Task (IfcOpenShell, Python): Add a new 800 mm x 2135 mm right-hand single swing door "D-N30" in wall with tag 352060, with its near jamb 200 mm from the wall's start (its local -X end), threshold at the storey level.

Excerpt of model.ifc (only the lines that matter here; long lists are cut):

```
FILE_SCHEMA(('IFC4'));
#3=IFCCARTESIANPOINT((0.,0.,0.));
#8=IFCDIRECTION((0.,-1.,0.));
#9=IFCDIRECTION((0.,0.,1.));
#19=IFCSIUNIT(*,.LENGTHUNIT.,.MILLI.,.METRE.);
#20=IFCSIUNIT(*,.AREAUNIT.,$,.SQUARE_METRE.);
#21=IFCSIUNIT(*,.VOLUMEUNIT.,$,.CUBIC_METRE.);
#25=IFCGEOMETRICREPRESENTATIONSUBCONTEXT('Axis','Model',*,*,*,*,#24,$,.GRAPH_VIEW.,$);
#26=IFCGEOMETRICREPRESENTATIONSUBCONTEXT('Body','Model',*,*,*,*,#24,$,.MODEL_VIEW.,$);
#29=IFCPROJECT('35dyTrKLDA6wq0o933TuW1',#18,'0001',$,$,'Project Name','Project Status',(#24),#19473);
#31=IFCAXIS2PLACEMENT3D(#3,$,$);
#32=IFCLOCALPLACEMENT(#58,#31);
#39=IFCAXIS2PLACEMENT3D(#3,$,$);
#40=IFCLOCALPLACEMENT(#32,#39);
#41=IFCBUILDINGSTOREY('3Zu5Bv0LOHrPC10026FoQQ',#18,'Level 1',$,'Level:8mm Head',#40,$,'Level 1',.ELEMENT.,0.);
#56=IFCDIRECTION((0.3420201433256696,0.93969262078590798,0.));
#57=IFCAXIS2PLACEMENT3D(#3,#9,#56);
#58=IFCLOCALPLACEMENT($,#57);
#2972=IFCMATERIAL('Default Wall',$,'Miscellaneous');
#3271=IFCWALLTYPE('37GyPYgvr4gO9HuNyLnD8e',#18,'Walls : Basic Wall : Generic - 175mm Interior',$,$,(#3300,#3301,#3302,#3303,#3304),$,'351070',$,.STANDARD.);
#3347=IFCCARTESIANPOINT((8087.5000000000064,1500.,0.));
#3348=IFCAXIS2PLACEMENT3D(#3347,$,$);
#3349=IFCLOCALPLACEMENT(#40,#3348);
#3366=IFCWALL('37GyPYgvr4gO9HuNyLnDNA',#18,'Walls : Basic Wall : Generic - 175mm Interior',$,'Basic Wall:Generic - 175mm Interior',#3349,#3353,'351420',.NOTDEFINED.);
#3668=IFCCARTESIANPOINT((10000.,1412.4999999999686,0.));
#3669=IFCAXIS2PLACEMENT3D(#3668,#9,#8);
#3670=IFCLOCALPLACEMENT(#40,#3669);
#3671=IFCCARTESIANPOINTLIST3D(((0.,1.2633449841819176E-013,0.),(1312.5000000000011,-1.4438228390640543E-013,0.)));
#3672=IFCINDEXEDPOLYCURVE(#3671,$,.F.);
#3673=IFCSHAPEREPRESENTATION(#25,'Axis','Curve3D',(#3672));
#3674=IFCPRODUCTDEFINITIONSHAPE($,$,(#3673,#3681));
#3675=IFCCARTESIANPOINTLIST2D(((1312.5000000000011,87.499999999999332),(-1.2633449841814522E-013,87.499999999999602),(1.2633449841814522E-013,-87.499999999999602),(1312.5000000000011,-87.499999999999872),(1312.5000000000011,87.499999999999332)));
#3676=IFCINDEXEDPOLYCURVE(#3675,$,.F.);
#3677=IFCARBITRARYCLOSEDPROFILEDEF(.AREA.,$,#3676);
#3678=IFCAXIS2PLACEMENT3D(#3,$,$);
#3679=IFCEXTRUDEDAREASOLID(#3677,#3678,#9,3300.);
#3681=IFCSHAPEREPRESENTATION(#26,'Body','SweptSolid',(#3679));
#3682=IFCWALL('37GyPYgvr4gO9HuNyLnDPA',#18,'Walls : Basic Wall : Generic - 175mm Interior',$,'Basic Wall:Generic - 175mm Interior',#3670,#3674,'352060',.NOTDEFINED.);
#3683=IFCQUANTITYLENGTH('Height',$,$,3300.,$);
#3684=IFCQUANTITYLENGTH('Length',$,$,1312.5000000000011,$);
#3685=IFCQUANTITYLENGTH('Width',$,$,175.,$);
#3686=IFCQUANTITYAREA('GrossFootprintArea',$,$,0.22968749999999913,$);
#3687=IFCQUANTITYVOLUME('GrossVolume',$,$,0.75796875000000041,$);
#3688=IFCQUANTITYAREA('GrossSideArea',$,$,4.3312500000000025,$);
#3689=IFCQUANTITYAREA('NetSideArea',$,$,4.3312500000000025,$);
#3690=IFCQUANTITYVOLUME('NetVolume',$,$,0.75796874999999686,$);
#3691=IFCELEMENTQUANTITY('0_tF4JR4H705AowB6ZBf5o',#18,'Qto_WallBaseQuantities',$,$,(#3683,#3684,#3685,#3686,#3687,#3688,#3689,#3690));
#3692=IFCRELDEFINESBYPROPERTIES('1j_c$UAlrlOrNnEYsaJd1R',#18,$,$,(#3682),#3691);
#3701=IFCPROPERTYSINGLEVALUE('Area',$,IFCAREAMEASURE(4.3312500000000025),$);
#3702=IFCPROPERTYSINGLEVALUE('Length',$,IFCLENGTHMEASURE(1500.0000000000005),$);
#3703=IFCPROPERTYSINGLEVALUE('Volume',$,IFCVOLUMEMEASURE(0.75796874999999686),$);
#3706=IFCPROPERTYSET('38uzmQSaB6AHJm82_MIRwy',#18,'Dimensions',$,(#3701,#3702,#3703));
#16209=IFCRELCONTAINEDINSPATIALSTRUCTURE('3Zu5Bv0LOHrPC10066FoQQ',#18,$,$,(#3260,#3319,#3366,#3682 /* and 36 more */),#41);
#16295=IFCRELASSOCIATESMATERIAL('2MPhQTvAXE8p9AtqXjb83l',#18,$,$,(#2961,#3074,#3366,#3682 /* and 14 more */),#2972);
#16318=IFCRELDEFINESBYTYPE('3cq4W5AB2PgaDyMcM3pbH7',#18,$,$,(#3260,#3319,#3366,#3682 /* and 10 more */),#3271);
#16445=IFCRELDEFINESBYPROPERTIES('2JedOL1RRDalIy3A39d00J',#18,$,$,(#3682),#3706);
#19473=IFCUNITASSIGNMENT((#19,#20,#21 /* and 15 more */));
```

```python
import numpy as np
import ifcopenshell
import ifcopenshell.api.feature
import ifcopenshell.api.geometry
import ifcopenshell.api.pset
import ifcopenshell.api.root
import ifcopenshell.api.spatial
import ifcopenshell.geom
import ifcopenshell.util.element
import ifcopenshell.util.placement
import ifcopenshell.util.representation
import ifcopenshell.util.shape
import ifcopenshell.util.unit

model = ifcopenshell.open("model.ifc")
unit_scale = ifcopenshell.util.unit.calculate_unit_scale(model)
area_scale = ifcopenshell.util.unit.calculate_unit_scale(model, "AREAUNIT")
volume_scale = ifcopenshell.util.unit.calculate_unit_scale(model, "VOLUMEUNIT")
settings = ifcopenshell.geom.settings()


def volume(element):
    """Net volume in cubic metres, openings subtracted."""
    shape = ifcopenshell.geom.create_shape(settings, element)
    return ifcopenshell.util.shape.get_volume(shape.geometry)


wall = model.by_guid("37GyPYgvr4gO9HuNyLnDPA")
storey = ifcopenshell.util.element.get_container(wall, ifc_class="IfcBuildingStorey")
context = ifcopenshell.util.representation.get_context(model, "Model", "Body", "MODEL_VIEW")
before = volume(wall)

width, height, from_end, sill = 0.8, 2.135, 0.2, 0.0  # metres

# The wall runs along its own X axis, and the end named is its -X end.
wall_shape = ifcopenshell.geom.create_shape(settings, wall)
x, y, z = ifcopenshell.util.shape.get_vertices(wall_shape.geometry).T
start = x.min() + from_end
face, thickness = float(y.min()), float(y.max() - y.min())
wall_matrix = ifcopenshell.util.placement.get_local_placement(wall.ObjectPlacement)
level = ifcopenshell.util.placement.get_local_placement(storey.ObjectPlacement)[2, 3]


def in_wall(x, y):
    """Placement at x, y metres in the wall's axes, at sill height."""
    matrix = wall_matrix.copy()
    matrix[:, 3] = wall_matrix @ np.array([x / unit_scale, y / unit_scale, 0.0, 1.0])
    matrix[2, 3] = level + sill / unit_scale
    return matrix


# Opening: a box that overshoots both wall faces by 50 mm.
opening = ifcopenshell.api.root.create_entity(model, ifc_class="IfcOpeningElement", predefined_type="OPENING")
box = ifcopenshell.api.geometry.add_wall_representation(
    model, context=context, length=width, height=height, thickness=thickness + 0.1
)
ifcopenshell.api.geometry.assign_representation(model, product=opening, representation=box)
ifcopenshell.api.geometry.edit_object_placement(model, product=opening, matrix=in_wall(start, face - 0.05), is_si=False)
ifcopenshell.api.feature.add_feature(model, feature=opening, element=wall)

door = ifcopenshell.api.root.create_entity(model, ifc_class="IfcDoor", name="D-N30", predefined_type="DOOR")
door.OverallWidth, door.OverallHeight = width / unit_scale, height / unit_scale
door.OperationType = "SINGLE_SWING_RIGHT"
body = ifcopenshell.api.geometry.add_door_representation(
    model,
    context=context,
    overall_width=door.OverallWidth,
    overall_height=door.OverallHeight,
    operation_type="SINGLE_SWING_RIGHT",
    lining_properties={"LiningDepth": thickness / unit_scale, "ThresholdDepth": thickness / unit_scale},
)
ifcopenshell.api.geometry.assign_representation(model, product=door, representation=body)
ifcopenshell.api.spatial.assign_container(model, products=[door], relating_structure=storey)
ifcopenshell.api.feature.add_filling(model, opening=opening, element=door)

# The lining spans the wall, so the door starts at the wall face.
ifcopenshell.api.geometry.edit_object_placement(model, product=door, matrix=in_wall(start, face), is_si=False)

after = volume(wall)

# Update the wall's stored quantities.
qto = model.by_id(ifcopenshell.util.element.get_pset(wall, "Qto_WallBaseQuantities", should_inherit=False)["id"])
ifcopenshell.api.pset.edit_qto(model, qto=qto, properties={
    "NetSideArea": after / thickness / area_scale,
    "NetVolume": after / volume_scale,
})
pset = model.by_id(ifcopenshell.util.element.get_pset(wall, "Dimensions", should_inherit=False)["id"])
ifcopenshell.api.pset.edit_pset(model, pset=pset, properties={
    "Area": model.create_entity("IfcAreaMeasure", after / thickness / area_scale),
    "Volume": model.create_entity("IfcVolumeMeasure", after / volume_scale),
})

print(f"wall volume {before:.3f} -> {after:.3f} m3")

model.write("model_v2.ifc")
```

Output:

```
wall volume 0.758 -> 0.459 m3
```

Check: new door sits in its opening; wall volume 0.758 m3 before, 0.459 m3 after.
